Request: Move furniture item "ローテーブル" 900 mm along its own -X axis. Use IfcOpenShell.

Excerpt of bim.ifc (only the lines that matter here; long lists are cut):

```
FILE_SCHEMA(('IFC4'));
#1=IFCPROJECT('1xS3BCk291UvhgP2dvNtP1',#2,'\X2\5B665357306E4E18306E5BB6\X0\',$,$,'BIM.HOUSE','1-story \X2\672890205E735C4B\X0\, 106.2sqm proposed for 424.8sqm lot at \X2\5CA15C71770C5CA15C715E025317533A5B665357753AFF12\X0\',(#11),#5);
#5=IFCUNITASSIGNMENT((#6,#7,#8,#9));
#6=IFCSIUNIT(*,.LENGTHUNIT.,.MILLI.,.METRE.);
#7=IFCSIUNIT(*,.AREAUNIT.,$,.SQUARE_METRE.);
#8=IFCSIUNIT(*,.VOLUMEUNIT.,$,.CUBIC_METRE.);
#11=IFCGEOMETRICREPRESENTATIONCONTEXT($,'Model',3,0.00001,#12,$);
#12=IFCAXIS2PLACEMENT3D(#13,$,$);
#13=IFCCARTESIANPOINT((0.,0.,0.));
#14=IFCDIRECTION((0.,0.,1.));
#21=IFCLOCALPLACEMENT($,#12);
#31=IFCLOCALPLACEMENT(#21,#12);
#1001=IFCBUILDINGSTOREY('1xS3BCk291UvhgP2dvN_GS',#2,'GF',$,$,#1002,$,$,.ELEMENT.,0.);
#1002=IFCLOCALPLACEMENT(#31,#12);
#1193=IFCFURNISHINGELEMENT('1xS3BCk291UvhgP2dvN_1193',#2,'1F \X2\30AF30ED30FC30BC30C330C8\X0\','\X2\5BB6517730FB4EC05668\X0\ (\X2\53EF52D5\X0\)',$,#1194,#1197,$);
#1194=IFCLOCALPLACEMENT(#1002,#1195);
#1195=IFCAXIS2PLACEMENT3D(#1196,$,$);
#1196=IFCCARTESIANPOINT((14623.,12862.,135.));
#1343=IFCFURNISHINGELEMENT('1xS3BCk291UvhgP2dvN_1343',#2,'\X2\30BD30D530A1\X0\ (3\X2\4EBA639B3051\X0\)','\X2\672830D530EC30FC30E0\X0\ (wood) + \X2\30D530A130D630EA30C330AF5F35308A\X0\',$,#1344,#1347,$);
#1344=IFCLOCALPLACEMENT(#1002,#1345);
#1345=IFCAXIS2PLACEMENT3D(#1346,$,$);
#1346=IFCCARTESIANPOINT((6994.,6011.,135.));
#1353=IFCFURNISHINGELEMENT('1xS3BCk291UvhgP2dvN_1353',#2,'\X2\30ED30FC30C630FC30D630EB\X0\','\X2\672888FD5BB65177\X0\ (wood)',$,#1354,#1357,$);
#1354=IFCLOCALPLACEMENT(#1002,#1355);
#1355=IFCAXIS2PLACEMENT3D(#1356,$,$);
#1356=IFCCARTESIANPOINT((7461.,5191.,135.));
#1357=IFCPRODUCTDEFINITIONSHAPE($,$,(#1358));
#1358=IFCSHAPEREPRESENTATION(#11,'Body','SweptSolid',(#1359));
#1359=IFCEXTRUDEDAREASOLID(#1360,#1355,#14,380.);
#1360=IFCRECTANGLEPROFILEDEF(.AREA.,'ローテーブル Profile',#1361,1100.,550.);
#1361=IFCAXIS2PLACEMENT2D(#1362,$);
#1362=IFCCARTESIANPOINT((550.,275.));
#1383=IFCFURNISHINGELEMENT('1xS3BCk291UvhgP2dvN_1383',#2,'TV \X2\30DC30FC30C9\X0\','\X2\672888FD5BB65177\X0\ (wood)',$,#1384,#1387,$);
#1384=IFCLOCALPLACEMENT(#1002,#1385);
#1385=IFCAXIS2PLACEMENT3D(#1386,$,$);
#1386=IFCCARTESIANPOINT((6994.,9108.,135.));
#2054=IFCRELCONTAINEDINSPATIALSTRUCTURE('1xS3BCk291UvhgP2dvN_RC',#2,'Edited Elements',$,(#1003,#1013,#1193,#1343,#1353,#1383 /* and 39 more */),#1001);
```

```python
import ifcopenshell
import ifcopenshell.api.geometry
import ifcopenshell.util.placement
import ifcopenshell.util.unit

model = ifcopenshell.open("bim.ifc")
unit_scale = ifcopenshell.util.unit.calculate_unit_scale(model)

item = model.by_guid("1xS3BCk291UvhgP2dvN_1353")
matrix = ifcopenshell.util.placement.get_local_placement(item.ObjectPlacement)
matrix[:3, 3] -= matrix[:3, 0] * 0.9 / unit_scale
ifcopenshell.api.geometry.edit_object_placement(model, product=item, matrix=matrix, is_si=False)

print(ifcopenshell.util.placement.get_local_placement(item.ObjectPlacement).round(3) + 0.0)

model.write("bim_v2.ifc")
```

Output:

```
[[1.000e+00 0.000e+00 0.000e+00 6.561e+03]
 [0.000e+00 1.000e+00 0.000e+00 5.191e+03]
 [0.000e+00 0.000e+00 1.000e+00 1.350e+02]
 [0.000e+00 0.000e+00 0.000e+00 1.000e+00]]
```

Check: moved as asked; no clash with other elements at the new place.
